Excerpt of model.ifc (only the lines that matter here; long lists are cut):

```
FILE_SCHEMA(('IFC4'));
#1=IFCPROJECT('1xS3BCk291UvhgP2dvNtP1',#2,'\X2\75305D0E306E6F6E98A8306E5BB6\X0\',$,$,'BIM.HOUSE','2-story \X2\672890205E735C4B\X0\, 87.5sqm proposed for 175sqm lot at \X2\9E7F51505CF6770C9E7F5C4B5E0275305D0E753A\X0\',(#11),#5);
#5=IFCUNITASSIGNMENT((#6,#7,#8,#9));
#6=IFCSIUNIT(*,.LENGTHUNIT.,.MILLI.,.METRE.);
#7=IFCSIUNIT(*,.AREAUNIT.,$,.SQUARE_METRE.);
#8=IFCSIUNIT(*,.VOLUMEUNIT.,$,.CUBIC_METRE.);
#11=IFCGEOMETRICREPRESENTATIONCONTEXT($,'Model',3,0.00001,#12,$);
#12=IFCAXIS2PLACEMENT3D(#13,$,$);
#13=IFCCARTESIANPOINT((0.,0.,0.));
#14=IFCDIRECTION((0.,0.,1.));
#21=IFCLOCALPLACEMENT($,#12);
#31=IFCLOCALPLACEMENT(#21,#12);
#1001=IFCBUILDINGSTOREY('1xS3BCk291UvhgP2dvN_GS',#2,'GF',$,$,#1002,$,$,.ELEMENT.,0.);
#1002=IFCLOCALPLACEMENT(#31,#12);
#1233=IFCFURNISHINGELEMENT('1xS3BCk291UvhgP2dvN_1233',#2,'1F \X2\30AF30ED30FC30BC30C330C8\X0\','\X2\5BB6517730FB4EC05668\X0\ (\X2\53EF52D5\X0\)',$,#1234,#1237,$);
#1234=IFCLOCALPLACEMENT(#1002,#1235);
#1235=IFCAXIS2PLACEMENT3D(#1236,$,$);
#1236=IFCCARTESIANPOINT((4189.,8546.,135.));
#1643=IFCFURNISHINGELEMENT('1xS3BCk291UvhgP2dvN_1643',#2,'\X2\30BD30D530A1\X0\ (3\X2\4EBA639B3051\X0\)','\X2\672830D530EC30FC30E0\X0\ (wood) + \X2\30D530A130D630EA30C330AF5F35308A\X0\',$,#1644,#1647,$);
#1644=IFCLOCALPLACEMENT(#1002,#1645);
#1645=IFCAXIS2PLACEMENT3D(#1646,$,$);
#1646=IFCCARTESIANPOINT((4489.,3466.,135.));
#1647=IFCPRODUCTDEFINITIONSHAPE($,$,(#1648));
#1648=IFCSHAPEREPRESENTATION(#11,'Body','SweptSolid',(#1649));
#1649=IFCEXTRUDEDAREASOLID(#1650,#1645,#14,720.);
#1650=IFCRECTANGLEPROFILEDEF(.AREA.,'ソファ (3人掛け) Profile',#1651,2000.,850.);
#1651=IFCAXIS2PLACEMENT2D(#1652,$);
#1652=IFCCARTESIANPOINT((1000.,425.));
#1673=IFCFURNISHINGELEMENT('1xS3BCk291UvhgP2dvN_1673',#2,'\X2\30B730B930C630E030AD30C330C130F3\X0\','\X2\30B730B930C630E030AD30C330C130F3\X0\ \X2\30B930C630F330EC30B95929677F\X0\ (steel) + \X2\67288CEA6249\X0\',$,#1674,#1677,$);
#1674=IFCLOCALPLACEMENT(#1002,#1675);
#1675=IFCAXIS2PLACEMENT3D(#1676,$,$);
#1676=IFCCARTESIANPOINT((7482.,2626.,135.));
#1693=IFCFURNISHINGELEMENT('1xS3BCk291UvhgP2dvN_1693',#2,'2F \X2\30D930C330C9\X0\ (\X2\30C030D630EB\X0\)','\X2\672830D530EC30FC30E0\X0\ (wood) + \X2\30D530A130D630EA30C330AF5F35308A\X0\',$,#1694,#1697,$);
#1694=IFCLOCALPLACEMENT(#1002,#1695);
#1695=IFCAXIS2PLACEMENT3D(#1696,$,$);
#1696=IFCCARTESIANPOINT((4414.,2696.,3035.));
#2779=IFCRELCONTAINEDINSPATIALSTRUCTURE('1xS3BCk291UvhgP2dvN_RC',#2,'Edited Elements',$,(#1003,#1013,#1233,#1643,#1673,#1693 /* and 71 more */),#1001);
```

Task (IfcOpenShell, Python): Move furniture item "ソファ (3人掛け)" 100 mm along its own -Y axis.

```python
import ifcopenshell
import ifcopenshell.api.geometry
import ifcopenshell.util.placement
import ifcopenshell.util.unit

model = ifcopenshell.open("model.ifc")
unit_scale = ifcopenshell.util.unit.calculate_unit_scale(model)

item = model.by_guid("1xS3BCk291UvhgP2dvN_1643")
matrix = ifcopenshell.util.placement.get_local_placement(item.ObjectPlacement)
matrix[:3, 3] -= matrix[:3, 1] * 0.1 / unit_scale
ifcopenshell.api.geometry.edit_object_placement(model, product=item, matrix=matrix, is_si=False)

print(ifcopenshell.util.placement.get_local_placement(item.ObjectPlacement).round(3) + 0.0)

model.write("model_updated.ifc")
```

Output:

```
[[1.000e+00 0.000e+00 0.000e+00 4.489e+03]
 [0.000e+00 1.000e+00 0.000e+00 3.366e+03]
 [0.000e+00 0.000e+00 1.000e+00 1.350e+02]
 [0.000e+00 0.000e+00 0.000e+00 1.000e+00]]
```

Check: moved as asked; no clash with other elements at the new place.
